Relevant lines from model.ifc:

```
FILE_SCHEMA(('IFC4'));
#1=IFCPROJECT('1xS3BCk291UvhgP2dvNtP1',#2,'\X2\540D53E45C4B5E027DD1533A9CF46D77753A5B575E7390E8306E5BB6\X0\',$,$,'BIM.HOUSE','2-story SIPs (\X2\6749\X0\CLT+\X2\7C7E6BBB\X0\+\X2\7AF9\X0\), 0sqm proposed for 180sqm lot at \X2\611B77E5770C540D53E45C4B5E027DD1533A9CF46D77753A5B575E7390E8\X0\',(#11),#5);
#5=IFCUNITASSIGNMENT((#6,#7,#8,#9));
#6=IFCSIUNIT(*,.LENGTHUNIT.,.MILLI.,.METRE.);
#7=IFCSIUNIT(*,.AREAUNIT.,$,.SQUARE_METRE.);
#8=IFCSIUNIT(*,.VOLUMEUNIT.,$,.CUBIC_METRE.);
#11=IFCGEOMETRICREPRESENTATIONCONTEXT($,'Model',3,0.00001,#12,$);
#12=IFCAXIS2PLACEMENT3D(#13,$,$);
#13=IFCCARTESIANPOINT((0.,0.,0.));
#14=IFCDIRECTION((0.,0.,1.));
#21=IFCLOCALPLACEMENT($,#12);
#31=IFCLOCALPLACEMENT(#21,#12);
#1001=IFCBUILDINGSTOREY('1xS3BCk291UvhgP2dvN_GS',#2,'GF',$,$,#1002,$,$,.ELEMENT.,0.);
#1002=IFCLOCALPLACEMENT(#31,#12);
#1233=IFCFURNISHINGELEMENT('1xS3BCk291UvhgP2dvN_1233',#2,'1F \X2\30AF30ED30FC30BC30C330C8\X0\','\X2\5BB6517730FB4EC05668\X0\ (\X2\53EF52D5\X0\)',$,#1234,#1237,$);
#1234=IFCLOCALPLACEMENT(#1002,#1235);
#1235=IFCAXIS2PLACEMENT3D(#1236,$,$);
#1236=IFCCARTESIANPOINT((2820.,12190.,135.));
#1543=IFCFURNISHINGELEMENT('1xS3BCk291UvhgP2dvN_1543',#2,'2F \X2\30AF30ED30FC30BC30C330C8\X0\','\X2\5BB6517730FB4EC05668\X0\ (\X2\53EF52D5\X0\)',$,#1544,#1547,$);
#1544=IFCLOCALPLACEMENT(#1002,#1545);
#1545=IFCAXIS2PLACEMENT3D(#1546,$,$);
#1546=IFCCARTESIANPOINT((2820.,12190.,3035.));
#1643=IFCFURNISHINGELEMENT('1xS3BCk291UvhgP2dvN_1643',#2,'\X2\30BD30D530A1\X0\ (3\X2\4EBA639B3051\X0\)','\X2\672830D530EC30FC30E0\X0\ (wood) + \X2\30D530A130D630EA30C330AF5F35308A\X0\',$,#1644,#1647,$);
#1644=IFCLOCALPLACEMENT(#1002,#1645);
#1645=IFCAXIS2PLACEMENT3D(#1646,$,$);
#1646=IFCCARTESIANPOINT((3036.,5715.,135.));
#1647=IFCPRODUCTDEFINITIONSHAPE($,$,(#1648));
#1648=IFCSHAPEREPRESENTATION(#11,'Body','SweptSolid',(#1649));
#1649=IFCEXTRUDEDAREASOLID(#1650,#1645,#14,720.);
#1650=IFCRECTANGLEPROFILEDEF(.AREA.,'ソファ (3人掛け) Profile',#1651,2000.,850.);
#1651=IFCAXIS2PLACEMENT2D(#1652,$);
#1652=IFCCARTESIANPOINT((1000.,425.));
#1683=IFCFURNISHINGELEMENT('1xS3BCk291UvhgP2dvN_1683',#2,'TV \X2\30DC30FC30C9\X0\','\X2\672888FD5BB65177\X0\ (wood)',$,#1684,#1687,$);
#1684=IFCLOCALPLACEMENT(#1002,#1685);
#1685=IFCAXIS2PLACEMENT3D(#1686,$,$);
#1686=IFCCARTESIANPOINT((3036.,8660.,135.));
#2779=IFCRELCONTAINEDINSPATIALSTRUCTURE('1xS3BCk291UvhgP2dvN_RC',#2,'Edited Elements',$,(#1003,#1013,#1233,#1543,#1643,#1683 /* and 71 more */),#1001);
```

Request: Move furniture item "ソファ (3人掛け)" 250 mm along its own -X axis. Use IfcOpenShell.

```python
import ifcopenshell
import ifcopenshell.api.geometry
import ifcopenshell.util.placement

model = ifcopenshell.open("model.ifc")

item = model.by_guid("1xS3BCk291UvhgP2dvN_1643")
matrix = ifcopenshell.util.placement.get_local_placement(item.ObjectPlacement)
matrix[:3, 3] -= matrix[:3, 0] * 250.0
ifcopenshell.api.geometry.edit_object_placement(model, product=item, matrix=matrix, is_si=False)

print(ifcopenshell.util.placement.get_local_placement(item.ObjectPlacement).round(3) + 0.0)

model.write("model_edited.ifc")
```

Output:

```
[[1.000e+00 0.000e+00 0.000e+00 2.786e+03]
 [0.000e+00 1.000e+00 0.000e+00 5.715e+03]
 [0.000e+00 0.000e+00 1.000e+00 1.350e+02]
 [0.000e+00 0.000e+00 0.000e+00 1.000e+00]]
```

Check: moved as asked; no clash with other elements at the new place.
